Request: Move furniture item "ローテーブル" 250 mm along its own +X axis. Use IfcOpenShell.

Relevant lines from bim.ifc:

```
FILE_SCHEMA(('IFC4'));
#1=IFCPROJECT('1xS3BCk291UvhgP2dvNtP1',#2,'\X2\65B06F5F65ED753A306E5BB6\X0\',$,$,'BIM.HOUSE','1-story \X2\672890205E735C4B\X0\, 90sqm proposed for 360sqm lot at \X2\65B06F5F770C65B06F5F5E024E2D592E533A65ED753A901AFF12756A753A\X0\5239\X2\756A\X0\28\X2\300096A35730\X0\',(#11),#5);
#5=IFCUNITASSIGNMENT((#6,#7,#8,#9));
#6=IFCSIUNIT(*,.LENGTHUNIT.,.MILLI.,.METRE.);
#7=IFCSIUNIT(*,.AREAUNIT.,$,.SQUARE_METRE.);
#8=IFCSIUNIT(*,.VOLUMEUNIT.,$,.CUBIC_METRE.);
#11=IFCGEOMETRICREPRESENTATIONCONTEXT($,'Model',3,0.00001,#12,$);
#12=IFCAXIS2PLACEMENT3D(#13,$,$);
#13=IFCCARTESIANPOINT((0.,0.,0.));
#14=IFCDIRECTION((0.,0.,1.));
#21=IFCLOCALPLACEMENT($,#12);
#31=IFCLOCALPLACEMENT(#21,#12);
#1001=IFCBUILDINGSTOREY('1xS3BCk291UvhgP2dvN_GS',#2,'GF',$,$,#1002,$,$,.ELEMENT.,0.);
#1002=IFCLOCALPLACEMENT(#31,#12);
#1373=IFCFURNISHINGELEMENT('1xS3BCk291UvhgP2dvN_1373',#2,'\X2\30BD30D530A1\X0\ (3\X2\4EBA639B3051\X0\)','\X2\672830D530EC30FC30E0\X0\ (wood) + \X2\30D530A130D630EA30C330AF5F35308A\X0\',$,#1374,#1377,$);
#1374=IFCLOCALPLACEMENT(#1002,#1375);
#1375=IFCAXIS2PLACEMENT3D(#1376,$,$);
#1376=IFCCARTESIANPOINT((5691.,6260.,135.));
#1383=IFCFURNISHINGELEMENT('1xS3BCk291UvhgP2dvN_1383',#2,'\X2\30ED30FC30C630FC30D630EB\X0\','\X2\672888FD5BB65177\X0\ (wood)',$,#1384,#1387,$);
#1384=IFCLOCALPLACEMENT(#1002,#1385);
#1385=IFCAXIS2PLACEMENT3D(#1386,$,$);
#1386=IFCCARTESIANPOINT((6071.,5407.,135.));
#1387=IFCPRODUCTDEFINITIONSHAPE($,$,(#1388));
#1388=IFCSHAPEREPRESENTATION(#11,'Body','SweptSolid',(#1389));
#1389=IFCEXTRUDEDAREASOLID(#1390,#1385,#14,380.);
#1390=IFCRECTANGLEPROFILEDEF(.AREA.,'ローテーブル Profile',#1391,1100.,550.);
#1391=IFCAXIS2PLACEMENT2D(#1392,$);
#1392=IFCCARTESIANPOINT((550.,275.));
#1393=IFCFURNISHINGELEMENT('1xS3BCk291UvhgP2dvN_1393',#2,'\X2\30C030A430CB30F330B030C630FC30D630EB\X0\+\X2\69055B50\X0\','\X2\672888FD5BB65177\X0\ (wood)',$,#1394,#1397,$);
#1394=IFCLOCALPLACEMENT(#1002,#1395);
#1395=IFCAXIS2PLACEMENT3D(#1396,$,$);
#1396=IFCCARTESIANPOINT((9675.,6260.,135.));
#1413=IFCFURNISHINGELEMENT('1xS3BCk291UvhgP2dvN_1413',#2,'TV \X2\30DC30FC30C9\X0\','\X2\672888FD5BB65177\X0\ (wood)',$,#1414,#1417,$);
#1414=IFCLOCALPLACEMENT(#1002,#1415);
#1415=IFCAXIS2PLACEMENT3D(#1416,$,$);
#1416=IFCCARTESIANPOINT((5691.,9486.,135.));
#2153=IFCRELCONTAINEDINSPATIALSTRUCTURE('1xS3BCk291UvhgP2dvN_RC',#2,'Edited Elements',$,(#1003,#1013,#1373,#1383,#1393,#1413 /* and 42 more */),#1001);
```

```python
import ifcopenshell
import ifcopenshell.api.geometry
import ifcopenshell.util.placement
import ifcopenshell.util.unit

model = ifcopenshell.open("bim.ifc")
unit_scale = ifcopenshell.util.unit.calculate_unit_scale(model)

item = model.by_guid("1xS3BCk291UvhgP2dvN_1383")
matrix = ifcopenshell.util.placement.get_local_placement(item.ObjectPlacement)
matrix[:3, 3] += matrix[:3, 0] * 0.25 / unit_scale
ifcopenshell.api.geometry.edit_object_placement(model, product=item, matrix=matrix, is_si=False)

print(ifcopenshell.util.placement.get_local_placement(item.ObjectPlacement).round(3) + 0.0)

model.write("bim_rev.ifc")
```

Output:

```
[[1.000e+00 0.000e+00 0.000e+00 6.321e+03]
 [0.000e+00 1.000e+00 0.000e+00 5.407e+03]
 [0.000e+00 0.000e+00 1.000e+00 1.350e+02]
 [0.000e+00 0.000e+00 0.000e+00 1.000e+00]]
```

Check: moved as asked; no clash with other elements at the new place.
